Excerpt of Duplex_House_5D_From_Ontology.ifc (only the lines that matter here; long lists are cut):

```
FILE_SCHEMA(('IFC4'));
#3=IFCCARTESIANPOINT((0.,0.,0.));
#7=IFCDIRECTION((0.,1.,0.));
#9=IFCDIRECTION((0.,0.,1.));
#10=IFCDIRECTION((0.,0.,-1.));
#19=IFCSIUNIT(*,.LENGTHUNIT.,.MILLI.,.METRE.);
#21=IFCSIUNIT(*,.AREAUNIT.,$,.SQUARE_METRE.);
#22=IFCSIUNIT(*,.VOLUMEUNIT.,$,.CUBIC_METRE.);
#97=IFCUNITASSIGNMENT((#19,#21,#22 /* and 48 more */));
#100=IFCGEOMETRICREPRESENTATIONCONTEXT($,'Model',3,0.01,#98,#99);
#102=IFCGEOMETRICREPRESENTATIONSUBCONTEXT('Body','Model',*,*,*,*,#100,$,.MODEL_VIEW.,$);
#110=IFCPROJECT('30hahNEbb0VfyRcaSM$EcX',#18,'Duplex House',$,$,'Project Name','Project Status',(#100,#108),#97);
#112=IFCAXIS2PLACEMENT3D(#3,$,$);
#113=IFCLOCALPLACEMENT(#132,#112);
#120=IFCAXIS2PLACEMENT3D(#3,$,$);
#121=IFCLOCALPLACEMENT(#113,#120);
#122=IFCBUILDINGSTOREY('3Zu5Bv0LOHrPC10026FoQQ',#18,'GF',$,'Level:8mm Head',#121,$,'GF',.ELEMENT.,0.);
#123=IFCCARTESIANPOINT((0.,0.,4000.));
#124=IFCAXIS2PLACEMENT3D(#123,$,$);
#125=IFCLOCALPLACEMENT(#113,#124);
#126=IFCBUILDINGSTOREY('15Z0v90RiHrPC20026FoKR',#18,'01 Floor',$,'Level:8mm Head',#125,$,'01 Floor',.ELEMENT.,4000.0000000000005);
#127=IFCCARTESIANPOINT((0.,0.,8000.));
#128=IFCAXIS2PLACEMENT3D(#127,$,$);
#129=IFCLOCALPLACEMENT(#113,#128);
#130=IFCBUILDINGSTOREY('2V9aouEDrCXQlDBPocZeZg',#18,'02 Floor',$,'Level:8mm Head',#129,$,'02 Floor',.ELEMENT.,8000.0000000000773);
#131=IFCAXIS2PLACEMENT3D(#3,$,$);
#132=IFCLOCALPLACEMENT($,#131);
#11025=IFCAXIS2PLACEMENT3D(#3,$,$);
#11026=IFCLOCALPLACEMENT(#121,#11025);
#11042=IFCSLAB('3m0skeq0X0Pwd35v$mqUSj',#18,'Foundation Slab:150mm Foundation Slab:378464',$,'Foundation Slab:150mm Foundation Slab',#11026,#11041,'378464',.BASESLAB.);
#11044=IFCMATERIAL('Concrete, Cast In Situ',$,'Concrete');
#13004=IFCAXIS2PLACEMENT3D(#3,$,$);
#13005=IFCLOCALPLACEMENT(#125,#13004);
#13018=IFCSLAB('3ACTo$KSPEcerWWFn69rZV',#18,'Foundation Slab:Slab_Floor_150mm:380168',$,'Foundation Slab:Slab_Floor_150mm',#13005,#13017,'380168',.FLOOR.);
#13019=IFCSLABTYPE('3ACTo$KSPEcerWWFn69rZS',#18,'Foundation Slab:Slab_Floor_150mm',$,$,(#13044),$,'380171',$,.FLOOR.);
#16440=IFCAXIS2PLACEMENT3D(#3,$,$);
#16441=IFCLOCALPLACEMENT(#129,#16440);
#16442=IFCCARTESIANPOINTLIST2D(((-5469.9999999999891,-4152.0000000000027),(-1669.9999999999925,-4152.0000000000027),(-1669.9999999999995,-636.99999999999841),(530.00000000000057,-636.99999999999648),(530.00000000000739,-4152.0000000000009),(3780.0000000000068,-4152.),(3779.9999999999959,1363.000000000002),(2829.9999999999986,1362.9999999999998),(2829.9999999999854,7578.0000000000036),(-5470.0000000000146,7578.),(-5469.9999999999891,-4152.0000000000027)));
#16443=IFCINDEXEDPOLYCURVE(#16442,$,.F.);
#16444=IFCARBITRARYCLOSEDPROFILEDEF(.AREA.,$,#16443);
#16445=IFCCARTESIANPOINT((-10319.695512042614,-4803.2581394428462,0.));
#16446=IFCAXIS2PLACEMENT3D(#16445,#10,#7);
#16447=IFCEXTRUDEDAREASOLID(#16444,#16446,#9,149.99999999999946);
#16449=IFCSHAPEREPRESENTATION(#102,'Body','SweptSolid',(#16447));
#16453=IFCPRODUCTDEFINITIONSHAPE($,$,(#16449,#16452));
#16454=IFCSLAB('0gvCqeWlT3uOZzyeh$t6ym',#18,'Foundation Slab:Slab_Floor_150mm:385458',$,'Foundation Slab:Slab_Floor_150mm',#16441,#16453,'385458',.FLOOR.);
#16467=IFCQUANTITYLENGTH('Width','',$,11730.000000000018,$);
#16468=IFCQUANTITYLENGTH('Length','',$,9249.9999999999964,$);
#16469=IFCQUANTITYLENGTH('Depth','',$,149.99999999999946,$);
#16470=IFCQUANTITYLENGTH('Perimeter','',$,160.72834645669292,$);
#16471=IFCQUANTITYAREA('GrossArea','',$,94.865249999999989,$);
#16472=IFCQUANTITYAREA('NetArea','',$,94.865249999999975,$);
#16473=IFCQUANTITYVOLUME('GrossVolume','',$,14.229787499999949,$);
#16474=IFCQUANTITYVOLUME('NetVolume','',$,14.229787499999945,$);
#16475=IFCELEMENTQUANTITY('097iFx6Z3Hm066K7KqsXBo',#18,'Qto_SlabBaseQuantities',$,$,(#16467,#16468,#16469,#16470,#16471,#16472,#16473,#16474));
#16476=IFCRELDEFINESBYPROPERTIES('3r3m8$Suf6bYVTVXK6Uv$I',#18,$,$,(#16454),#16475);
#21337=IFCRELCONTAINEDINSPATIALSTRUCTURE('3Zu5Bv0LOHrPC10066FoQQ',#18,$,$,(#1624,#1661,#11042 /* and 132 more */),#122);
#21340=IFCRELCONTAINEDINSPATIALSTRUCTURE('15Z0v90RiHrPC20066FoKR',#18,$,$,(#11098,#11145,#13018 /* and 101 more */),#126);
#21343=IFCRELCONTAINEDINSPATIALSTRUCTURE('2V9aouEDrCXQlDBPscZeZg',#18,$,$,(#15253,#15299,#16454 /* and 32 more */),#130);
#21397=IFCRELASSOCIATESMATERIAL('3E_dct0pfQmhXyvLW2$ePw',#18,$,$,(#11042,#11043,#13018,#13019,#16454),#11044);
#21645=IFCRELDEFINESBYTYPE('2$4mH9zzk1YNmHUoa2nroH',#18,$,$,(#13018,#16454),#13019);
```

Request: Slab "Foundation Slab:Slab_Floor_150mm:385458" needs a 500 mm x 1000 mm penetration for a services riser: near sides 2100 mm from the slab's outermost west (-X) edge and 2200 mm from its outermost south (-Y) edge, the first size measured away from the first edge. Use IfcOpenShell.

```python
import numpy as np
import ifcopenshell
import ifcopenshell.api.feature
import ifcopenshell.api.geometry
import ifcopenshell.api.pset
import ifcopenshell.api.root
import ifcopenshell.geom
import ifcopenshell.util.element
import ifcopenshell.util.placement
import ifcopenshell.util.representation
import ifcopenshell.util.shape
import ifcopenshell.util.unit

model = ifcopenshell.open("Duplex_House_5D_From_Ontology.ifc")
unit_scale = ifcopenshell.util.unit.calculate_unit_scale(model)
area_scale = ifcopenshell.util.unit.calculate_unit_scale(model, "AREAUNIT")
volume_scale = ifcopenshell.util.unit.calculate_unit_scale(model, "VOLUMEUNIT")
settings = ifcopenshell.geom.settings()


def volume(element):
    """Net volume in cubic metres, openings subtracted."""
    shape = ifcopenshell.geom.create_shape(settings, element)
    return ifcopenshell.util.shape.get_volume(shape.geometry)


slab = model.by_id(16454)
before = volume(slab)

# Extent in the slab's own axes, in metres. The edges named are its -X and -Y sides.
slab_shape = ifcopenshell.geom.create_shape(settings, slab)
vertices = ifcopenshell.util.shape.get_vertices(slab_shape.geometry)
x_min, y_min, bottom = vertices.min(axis=0)
top = vertices[:, 2].max()

opening = ifcopenshell.api.root.create_entity(model, ifc_class="IfcOpeningElement", name="Services riser opening", predefined_type="OPENING")
context = ifcopenshell.util.representation.get_context(model, "Model", "Body", "MODEL_VIEW")
width, depth = 0.5, 1
outline = [(0.0, 0.0), (width, 0.0), (width, depth), (0.0, depth), (0.0, 0.0)]
# Overshoot both faces by 50 mm so the cut is clean.
shape = ifcopenshell.api.geometry.add_slab_representation(
    model, context=context, depth=top - bottom + 0.1, polyline=outline
)
ifcopenshell.api.geometry.assign_representation(model, product=opening, representation=shape)

matrix = ifcopenshell.util.placement.get_local_placement(slab.ObjectPlacement)
matrix[:, 3] = matrix @ np.append(np.array([x_min + 2.1, y_min + 2.2, bottom - 0.05]) / unit_scale, 1.0)
ifcopenshell.api.geometry.edit_object_placement(model, product=opening, matrix=matrix, is_si=False)
ifcopenshell.api.feature.add_feature(model, feature=opening, element=slab)

after = volume(slab)

# Update the slab's stored quantities.
qto = model.by_id(ifcopenshell.util.element.get_pset(slab, "Qto_SlabBaseQuantities", should_inherit=False)["id"])
ifcopenshell.api.pset.edit_qto(model, qto=qto, properties={
    "NetArea": after / (top - bottom) / area_scale,
    "NetVolume": after / volume_scale,
})

print(f"slab volume {before:.3f} -> {after:.3f} m3")

model.write("Duplex_House_5D_From_Ontology_edited.ifc")
```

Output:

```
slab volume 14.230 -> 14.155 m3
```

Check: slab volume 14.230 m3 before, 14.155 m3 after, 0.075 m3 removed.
